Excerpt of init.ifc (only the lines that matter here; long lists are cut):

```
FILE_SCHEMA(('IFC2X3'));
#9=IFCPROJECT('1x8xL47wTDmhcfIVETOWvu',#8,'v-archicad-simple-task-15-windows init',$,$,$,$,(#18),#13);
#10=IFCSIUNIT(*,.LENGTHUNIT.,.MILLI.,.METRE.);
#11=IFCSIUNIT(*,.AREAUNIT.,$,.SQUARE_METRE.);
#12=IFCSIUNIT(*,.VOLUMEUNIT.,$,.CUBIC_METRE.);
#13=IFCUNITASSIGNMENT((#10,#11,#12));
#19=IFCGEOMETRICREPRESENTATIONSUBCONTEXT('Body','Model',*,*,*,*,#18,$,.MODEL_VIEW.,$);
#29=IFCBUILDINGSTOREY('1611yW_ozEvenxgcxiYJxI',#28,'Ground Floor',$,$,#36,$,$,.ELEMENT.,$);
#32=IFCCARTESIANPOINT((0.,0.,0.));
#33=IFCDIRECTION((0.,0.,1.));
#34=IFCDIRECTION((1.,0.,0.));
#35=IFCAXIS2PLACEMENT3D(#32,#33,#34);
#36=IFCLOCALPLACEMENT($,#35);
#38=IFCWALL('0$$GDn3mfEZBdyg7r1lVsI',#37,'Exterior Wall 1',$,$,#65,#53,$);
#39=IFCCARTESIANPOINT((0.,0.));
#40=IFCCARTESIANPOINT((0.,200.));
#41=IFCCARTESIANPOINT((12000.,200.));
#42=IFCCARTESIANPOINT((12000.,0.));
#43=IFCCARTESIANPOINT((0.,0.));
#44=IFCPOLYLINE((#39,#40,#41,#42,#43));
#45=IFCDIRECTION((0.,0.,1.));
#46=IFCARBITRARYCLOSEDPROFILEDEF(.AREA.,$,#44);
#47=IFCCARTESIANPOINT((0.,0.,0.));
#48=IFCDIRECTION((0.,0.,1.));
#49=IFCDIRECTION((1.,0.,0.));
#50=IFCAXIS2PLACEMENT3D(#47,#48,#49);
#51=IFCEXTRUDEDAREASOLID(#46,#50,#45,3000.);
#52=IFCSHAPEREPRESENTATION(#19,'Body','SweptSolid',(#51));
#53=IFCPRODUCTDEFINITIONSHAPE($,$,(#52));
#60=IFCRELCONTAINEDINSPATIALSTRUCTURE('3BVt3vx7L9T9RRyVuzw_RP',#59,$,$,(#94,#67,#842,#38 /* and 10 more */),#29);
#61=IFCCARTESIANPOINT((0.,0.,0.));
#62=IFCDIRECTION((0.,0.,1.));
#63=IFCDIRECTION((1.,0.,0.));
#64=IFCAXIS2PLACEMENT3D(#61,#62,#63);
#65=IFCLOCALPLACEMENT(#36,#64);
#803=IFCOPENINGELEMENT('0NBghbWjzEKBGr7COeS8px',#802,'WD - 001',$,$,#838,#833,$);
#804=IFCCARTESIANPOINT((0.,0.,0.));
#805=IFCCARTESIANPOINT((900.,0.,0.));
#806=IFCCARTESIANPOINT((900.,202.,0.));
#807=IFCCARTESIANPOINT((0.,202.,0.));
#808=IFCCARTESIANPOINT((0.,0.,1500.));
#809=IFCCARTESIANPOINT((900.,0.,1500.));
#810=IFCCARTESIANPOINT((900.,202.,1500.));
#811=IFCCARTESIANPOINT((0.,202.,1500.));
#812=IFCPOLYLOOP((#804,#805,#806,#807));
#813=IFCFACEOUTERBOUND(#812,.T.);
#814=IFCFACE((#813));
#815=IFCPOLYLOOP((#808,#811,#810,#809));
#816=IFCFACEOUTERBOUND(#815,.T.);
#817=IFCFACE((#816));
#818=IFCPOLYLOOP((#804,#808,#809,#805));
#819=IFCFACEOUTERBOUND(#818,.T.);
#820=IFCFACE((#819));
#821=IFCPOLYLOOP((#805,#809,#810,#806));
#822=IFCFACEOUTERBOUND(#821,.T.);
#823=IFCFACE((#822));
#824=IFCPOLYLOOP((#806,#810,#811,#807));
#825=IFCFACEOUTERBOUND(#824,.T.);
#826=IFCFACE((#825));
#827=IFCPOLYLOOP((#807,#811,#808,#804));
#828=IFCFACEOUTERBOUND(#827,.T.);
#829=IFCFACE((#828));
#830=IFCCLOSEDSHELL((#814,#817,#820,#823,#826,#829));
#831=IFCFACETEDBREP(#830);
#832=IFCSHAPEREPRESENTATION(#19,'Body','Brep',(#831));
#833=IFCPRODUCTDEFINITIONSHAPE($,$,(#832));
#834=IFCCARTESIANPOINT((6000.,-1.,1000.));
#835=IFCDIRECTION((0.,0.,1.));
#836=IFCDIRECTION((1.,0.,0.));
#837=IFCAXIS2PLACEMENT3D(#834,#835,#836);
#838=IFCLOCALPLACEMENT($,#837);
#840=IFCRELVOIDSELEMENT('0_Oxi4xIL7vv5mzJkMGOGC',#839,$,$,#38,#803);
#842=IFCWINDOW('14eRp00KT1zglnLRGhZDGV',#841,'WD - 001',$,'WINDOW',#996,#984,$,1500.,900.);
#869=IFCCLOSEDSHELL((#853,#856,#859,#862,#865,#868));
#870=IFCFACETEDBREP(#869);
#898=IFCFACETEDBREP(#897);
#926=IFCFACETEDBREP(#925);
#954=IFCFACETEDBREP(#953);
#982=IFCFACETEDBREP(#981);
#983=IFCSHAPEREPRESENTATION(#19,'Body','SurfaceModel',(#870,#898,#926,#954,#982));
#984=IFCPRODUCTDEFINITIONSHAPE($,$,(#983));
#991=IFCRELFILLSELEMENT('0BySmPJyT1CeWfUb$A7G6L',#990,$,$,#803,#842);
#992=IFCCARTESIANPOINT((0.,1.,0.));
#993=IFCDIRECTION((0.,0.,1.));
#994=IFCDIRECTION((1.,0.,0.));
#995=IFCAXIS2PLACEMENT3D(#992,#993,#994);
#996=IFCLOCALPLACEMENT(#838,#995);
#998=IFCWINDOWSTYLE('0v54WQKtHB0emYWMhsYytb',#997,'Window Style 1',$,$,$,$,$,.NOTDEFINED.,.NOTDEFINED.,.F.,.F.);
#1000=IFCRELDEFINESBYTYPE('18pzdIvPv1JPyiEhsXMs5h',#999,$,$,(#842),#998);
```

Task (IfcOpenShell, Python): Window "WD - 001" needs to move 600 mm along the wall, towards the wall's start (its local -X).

```python
import ifcopenshell
import ifcopenshell.api.geometry
import ifcopenshell.util.placement
import ifcopenshell.util.unit

model = ifcopenshell.open("init.ifc")
unit_scale = ifcopenshell.util.unit.calculate_unit_scale(model)

window = model.by_id(842)
opening = window.FillsVoids[0].RelatingOpeningElement
wall = opening.VoidsElements[0].RelatingBuildingElement

wall_matrix = ifcopenshell.util.placement.get_local_placement(wall.ObjectPlacement)
shift = wall_matrix[:3, 0] * -0.6 / unit_scale
before = ifcopenshell.util.placement.get_local_placement(window.ObjectPlacement)[:3, 3].copy()

# The window is placed relative to its opening, so it follows when the opening moves.
matrix = ifcopenshell.util.placement.get_local_placement(opening.ObjectPlacement)
matrix[:3, 3] += shift
ifcopenshell.api.geometry.edit_object_placement(
    model, product=opening, matrix=matrix, is_si=False, should_transform_children=True
)

after = ifcopenshell.util.placement.get_local_placement(window.ObjectPlacement)[:3, 3]
print("window moved by", (after - before).round(3) + 0.0)

model.write("init_edited.ifc")
```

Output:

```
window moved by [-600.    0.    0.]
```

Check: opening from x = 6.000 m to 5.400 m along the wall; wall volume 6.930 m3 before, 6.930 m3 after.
